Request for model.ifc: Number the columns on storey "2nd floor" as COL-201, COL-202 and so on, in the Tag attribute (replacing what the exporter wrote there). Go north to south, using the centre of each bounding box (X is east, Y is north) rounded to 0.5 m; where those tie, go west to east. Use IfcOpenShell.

First a look at what the model holds.

```python
import ifcopenshell
import ifcopenshell.util.element
import ifcopenshell.util.placement

model = ifcopenshell.open("model.ifc")
print(model.schema)
storey = next(s for s in model.by_type("IfcBuildingStorey") if s.Name == "2nd floor")
columns = [e for e in ifcopenshell.util.element.get_decomposition(storey) if e.is_a("IfcColumn")]
for e in sorted(columns, key=lambda e: e.id()):
    origin = ifcopenshell.util.placement.get_local_placement(e.ObjectPlacement)[:3, 3]
    print(e.id(), e.Tag, e.Name, origin.round(2) + 0.0, sep=" | ")
```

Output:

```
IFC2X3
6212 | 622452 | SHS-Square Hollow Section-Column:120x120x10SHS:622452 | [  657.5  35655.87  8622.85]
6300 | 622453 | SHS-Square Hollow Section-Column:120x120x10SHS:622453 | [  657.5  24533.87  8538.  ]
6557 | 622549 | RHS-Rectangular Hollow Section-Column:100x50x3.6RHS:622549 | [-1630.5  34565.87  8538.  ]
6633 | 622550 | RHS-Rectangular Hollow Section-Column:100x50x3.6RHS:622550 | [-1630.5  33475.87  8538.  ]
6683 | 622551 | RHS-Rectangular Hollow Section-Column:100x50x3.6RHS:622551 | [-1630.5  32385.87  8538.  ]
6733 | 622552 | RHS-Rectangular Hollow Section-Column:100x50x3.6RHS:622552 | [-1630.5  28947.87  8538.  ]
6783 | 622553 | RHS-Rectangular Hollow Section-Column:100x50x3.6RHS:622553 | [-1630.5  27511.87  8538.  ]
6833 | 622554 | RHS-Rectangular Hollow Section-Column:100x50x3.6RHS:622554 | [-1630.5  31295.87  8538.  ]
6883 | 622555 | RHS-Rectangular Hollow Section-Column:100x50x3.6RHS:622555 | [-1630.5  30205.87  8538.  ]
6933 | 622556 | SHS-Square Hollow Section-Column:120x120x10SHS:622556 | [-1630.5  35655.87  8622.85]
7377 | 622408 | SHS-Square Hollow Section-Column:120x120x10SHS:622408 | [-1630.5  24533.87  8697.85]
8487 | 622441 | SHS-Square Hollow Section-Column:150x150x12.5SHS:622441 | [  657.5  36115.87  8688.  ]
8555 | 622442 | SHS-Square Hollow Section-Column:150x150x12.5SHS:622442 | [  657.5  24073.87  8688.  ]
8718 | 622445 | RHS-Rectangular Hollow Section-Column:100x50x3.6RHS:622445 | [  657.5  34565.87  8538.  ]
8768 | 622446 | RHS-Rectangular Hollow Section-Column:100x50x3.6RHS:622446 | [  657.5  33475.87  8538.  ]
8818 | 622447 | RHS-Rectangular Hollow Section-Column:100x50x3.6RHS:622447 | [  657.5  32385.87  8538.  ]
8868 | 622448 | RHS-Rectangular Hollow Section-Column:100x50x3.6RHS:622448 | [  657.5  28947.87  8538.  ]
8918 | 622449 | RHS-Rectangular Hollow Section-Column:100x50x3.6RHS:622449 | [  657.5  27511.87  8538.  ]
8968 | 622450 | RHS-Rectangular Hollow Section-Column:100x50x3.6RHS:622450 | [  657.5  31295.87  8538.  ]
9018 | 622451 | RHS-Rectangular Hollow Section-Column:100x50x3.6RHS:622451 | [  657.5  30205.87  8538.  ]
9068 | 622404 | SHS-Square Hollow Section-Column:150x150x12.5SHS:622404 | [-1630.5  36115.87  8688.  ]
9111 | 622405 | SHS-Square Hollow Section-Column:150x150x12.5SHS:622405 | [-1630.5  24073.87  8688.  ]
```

```python
import ifcopenshell
import ifcopenshell.geom
import ifcopenshell.util.element
import ifcopenshell.util.shape

model = ifcopenshell.open("model.ifc")
settings = ifcopenshell.geom.settings()
settings.set("use-world-coords", True)


def centre(element):
    shape = ifcopenshell.geom.create_shape(settings, element)
    return ifcopenshell.util.shape.get_bbox_centroid(shape.geometry)


storey = next(s for s in model.by_type("IfcBuildingStorey") if s.Name == "2nd floor")
columns = [e for e in ifcopenshell.util.element.get_decomposition(storey) if e.is_a("IfcColumn")]

# Insertion points can sit at a corner or the storey origin, so sort by the geometry (in metres).
centres = {e: centre(e) for e in columns}
columns.sort(key=lambda e: (-round(centres[e][1] / 0.5), centres[e][0]))

for i, e in enumerate(columns, start=1):
    number = f"COL-2{i:02d}"
    e.Tag = number
    print(e.id(), number)

model.write("model_edited.ifc")
```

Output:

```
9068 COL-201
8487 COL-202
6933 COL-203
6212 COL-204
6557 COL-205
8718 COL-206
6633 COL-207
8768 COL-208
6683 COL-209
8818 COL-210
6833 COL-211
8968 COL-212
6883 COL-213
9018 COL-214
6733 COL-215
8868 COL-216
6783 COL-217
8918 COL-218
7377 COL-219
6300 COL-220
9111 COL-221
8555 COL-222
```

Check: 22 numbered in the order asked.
